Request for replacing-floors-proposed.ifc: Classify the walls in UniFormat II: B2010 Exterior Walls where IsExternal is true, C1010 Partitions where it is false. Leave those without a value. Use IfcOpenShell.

First a look at what the model holds.

```python
import ifcopenshell
import ifcopenshell.util.element

model = ifcopenshell.open("replacing-floors-proposed.ifc")
print(model.schema)
print("classifications:", [c.Name for c in model.by_type("IfcClassification")])
values = [ifcopenshell.util.element.get_pset(e, "Pset_WallCommon", "IsExternal") for e in model.by_type("IfcWall")]
for value in (True, False, None):
    print("IsExternal", value, values.count(value))
```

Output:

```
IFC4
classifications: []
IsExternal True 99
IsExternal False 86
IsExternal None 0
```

```python
import ifcopenshell
import ifcopenshell.api.classification
import ifcopenshell.util.element

model = ifcopenshell.open("replacing-floors-proposed.ifc")

system = ifcopenshell.api.classification.add_classification(model, classification="UniFormat II")

walls = model.by_type("IfcWall")
external = {e: ifcopenshell.util.element.get_pset(e, "Pset_WallCommon", "IsExternal") for e in walls}
for flag, code, name in ((True, "B2010", "Exterior Walls"), (False, "C1010", "Partitions")):
    products = [e for e in walls if external[e] is flag]
    ifcopenshell.api.classification.add_reference(
        model, products=products, classification=system, identification=code, name=name
    )
    print(code, len(products))

model.write("replacing-floors-proposed_edited.ifc")
```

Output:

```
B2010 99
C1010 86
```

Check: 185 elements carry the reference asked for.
